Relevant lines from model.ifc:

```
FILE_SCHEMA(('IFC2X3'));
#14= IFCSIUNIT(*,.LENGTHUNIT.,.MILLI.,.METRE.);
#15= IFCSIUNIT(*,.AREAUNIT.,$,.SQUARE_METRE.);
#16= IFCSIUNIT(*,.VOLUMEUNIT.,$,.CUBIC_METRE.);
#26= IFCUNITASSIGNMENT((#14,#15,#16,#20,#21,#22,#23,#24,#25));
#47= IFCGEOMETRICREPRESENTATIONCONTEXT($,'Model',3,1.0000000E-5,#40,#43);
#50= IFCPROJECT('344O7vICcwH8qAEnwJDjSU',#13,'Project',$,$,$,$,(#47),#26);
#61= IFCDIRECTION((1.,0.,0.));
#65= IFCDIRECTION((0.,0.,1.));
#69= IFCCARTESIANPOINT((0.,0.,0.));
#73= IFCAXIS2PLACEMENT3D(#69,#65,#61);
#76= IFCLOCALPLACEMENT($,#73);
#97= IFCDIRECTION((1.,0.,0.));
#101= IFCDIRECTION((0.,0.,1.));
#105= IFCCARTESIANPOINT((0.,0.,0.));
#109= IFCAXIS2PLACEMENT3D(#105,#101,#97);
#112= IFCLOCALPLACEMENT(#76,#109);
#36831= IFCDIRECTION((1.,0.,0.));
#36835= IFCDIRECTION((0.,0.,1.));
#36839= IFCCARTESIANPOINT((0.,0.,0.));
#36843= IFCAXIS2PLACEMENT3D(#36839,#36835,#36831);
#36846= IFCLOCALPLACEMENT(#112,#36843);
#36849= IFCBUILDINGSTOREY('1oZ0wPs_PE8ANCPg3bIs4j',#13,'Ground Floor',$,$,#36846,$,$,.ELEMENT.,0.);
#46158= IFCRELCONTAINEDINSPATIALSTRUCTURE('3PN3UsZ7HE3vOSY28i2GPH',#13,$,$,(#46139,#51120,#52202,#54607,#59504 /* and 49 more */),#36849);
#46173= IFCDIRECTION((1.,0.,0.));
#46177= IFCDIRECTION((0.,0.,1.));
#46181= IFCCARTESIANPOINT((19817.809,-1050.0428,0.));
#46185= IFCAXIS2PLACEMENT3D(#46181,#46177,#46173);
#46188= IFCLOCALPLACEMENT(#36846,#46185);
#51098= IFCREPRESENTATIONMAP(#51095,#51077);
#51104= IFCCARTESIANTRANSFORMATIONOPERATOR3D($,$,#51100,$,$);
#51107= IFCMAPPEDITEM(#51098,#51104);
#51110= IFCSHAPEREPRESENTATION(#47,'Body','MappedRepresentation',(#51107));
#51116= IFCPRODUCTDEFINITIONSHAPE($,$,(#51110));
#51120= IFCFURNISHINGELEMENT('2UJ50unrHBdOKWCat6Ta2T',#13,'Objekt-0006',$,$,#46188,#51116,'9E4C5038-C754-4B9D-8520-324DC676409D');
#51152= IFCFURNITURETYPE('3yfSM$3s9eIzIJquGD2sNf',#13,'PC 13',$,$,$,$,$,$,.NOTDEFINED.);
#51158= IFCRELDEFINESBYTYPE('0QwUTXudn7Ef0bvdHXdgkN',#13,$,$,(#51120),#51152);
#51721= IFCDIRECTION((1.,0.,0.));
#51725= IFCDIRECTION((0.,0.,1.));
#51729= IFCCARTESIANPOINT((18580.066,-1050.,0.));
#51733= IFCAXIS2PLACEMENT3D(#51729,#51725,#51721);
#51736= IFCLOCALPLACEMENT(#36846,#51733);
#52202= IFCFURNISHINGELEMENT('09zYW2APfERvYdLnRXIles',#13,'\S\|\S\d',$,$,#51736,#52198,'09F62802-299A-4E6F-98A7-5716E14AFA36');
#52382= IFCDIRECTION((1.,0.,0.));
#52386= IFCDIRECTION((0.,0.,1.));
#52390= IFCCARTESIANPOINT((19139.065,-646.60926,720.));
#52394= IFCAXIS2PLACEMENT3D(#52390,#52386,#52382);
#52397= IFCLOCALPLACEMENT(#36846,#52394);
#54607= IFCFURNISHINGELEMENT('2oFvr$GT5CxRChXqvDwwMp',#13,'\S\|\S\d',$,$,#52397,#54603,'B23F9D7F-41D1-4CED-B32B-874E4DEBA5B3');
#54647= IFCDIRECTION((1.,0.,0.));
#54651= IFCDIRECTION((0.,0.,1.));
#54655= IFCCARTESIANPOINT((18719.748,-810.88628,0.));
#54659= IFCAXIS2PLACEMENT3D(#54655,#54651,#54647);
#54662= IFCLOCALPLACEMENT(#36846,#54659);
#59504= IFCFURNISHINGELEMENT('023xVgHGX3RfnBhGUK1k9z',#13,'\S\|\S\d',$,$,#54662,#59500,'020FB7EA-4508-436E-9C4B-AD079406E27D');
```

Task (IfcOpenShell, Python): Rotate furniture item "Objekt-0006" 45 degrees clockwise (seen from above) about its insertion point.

```python
import ifcopenshell
import ifcopenshell.api.geometry
import ifcopenshell.util.placement

model = ifcopenshell.open("model.ifc")

item = model.by_guid("2UJ50unrHBdOKWCat6Ta2T")
matrix = ifcopenshell.util.placement.get_local_placement(item.ObjectPlacement)
matrix = matrix @ ifcopenshell.util.placement.rotation(-45, "Z")
ifcopenshell.api.geometry.edit_object_placement(model, product=item, matrix=matrix, is_si=False)

print(ifcopenshell.util.placement.get_local_placement(item.ObjectPlacement).round(3) + 0.0)

model.write("model_edited.ifc")
```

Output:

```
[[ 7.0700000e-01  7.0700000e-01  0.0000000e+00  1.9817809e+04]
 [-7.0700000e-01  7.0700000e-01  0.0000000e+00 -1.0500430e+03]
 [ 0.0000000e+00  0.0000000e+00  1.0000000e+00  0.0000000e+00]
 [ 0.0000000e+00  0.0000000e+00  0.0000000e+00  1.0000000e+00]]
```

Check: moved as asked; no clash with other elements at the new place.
